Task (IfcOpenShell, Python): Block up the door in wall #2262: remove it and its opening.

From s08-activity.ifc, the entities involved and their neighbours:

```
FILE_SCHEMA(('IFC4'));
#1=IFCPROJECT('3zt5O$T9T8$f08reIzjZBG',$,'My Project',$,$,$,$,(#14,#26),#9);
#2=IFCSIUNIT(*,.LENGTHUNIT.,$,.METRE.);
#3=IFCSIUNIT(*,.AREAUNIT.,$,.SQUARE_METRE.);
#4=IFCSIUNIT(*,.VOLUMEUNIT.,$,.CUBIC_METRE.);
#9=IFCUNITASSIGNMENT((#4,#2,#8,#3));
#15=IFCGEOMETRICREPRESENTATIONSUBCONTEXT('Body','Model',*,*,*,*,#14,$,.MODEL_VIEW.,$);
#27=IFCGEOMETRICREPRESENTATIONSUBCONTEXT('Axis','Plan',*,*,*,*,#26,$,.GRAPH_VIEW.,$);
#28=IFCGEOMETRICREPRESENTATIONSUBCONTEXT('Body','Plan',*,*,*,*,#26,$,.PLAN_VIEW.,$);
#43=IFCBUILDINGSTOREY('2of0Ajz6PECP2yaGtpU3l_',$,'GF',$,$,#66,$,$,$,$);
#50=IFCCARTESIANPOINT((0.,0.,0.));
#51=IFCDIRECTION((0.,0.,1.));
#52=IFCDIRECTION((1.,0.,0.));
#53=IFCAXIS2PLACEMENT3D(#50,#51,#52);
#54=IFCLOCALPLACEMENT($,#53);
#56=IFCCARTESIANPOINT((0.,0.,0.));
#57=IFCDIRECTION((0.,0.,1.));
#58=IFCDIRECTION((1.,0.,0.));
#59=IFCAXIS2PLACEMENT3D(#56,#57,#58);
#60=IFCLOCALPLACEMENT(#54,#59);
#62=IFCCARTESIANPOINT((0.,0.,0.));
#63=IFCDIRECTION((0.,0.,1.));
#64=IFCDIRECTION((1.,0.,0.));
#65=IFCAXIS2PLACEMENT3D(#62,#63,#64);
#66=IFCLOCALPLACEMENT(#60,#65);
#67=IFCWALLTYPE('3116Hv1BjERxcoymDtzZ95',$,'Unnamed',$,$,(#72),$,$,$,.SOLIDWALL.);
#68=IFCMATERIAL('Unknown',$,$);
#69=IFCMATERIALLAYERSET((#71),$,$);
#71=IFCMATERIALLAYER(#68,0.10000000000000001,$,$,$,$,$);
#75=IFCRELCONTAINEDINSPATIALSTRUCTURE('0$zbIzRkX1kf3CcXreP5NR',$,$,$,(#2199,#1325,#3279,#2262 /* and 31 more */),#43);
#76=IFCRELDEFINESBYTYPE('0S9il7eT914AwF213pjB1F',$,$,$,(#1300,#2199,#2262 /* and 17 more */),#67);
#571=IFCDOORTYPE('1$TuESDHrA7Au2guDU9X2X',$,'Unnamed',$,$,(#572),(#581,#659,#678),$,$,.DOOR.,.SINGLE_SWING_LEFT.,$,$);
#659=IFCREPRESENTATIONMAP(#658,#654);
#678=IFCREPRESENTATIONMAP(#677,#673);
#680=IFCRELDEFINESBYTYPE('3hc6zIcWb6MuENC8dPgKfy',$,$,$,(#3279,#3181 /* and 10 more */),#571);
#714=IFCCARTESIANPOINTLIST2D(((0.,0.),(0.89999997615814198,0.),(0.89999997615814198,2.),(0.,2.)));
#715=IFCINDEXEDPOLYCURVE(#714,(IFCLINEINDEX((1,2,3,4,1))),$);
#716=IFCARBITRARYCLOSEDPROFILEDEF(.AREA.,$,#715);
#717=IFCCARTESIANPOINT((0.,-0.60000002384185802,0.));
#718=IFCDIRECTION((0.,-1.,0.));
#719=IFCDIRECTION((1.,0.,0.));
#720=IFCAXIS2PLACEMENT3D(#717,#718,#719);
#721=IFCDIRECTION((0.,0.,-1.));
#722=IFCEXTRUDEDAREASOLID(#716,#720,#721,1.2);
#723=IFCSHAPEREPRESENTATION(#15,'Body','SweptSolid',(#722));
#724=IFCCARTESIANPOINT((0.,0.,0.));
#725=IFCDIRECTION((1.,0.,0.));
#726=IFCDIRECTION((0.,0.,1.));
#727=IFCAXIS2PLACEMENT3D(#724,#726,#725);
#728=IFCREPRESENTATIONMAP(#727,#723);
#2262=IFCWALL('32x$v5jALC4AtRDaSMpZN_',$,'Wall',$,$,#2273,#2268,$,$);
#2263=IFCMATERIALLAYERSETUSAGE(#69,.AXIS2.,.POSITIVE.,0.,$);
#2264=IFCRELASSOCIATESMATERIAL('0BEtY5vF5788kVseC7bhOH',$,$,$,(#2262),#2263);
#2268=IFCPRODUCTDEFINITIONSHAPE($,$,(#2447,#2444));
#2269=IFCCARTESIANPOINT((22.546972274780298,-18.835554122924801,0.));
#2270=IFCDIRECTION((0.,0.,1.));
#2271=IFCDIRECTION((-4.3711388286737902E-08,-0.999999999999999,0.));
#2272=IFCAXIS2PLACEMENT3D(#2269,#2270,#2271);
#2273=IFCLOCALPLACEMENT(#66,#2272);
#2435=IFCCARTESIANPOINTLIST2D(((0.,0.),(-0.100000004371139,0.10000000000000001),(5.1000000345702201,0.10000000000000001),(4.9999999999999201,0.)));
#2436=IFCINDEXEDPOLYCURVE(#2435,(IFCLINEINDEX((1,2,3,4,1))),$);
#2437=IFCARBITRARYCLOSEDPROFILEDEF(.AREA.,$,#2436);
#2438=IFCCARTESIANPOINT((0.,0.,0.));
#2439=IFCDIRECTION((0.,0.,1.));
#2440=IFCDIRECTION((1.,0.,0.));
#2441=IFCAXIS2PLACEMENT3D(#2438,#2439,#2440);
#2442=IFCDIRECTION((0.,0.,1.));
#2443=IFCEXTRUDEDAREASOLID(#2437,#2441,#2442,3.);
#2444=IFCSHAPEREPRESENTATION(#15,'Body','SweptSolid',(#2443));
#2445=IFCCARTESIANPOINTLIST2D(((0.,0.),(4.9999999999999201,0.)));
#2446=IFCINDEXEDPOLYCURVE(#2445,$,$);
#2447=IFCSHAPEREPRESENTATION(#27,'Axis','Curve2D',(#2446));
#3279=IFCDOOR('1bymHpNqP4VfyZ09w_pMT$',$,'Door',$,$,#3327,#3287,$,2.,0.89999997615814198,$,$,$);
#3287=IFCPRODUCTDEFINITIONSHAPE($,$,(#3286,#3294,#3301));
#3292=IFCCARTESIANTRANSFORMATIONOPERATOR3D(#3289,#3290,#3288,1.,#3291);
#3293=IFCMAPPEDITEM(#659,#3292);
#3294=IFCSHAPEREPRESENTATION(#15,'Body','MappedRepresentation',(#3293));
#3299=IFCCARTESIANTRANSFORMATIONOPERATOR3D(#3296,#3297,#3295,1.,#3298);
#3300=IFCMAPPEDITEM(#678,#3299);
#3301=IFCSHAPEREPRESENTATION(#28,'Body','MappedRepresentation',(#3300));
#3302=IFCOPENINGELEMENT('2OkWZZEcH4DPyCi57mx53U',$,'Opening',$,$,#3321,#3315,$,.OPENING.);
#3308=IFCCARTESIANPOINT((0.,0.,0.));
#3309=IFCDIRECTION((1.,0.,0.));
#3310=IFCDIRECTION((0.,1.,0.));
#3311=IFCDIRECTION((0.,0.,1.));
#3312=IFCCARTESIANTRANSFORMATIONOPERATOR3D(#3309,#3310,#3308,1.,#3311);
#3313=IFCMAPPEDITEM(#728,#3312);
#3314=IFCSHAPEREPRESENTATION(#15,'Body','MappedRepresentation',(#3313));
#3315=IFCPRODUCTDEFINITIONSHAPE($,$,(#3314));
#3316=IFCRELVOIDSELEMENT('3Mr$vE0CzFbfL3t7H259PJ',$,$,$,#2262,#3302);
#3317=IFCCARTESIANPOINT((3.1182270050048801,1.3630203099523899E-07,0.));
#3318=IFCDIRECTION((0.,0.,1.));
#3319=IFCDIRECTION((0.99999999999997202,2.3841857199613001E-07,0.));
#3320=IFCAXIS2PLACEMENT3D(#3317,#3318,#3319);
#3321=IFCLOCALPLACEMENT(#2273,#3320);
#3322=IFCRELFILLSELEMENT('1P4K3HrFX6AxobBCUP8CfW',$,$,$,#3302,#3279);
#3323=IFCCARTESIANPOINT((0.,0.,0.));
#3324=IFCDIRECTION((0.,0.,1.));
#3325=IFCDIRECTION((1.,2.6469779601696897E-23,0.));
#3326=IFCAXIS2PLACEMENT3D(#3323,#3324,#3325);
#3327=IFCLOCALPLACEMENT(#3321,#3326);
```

```python
import ifcopenshell
import ifcopenshell.api.feature
import ifcopenshell.api.root
import ifcopenshell.geom
import ifcopenshell.util.shape

model = ifcopenshell.open("s08-activity.ifc")
settings = ifcopenshell.geom.settings()


def volume(element):
    """Net volume in cubic metres, openings subtracted."""
    shape = ifcopenshell.geom.create_shape(settings, element)
    return ifcopenshell.util.shape.get_volume(shape.geometry)


door = model.by_id(3279)
opening = door.FillsVoids[0].RelatingOpeningElement
wall = opening.VoidsElements[0].RelatingBuildingElement
before = volume(wall)

ifcopenshell.api.root.remove_product(model, product=door)
ifcopenshell.api.feature.remove_feature(model, feature=opening)

after = volume(wall)

print(f"wall volume {before:.3f} -> {after:.3f} m3")

model.write("s08-activity_updated.ifc")
```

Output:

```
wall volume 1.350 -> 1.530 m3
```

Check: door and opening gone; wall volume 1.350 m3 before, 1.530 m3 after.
